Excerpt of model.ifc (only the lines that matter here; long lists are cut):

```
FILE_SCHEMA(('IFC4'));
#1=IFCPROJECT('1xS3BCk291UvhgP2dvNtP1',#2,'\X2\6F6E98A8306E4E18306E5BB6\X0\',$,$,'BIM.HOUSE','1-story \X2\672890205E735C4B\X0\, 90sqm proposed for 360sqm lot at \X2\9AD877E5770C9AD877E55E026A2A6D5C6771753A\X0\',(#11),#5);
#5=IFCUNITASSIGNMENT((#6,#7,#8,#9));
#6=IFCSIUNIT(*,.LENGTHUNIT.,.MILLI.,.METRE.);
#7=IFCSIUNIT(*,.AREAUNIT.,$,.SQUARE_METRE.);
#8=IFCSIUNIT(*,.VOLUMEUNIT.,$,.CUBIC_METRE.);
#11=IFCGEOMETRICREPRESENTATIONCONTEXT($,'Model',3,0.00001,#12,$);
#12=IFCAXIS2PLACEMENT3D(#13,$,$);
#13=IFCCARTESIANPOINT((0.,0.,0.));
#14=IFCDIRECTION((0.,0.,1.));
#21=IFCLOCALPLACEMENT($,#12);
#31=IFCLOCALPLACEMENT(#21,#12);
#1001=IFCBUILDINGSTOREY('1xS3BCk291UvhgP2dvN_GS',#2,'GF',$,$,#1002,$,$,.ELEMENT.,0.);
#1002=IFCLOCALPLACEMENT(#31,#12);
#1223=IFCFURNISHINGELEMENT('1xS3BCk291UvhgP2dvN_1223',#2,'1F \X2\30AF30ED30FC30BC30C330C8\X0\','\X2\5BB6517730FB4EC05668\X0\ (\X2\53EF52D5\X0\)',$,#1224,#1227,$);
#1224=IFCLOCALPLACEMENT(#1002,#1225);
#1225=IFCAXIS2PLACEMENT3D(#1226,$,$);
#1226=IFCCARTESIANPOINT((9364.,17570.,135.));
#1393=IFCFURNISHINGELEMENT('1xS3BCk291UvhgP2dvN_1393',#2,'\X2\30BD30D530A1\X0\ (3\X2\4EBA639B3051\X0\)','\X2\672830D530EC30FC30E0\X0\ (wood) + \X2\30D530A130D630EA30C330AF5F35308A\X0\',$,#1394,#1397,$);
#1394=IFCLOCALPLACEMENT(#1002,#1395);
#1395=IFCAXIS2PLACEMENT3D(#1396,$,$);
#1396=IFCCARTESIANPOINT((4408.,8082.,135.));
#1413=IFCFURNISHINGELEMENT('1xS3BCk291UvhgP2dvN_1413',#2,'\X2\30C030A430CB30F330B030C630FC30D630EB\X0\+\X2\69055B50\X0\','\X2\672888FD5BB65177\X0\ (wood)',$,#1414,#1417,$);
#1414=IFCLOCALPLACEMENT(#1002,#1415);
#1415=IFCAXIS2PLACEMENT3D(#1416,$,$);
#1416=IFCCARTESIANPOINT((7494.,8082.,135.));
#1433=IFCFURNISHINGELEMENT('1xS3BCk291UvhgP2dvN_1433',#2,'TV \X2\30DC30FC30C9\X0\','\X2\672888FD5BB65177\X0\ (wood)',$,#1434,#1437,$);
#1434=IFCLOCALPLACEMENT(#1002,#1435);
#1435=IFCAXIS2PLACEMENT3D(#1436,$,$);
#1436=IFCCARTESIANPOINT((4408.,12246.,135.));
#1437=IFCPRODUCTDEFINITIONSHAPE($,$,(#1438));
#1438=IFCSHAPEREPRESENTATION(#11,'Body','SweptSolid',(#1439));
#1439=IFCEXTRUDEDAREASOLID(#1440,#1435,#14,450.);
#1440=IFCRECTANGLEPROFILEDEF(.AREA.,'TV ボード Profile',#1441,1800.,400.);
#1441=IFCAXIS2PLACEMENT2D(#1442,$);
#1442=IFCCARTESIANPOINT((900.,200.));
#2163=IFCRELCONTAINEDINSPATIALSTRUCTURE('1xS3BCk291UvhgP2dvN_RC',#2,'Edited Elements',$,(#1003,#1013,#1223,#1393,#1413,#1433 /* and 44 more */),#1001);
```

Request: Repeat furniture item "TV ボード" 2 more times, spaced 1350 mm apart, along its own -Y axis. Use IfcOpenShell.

```python
import ifcopenshell
import ifcopenshell.api.geometry
import ifcopenshell.api.root
import ifcopenshell.util.element
import ifcopenshell.util.placement

model = ifcopenshell.open("model.ifc")


def reuse_history(source, copy):
    """copy_class also copies each property set's owner history, people and application; keep the originals."""
    for rel in copy.IsDefinedBy:
        if rel.is_a("IfcRelDefinesByProperties") and (history := rel.RelatingPropertyDefinition.OwnerHistory):
            rel.RelatingPropertyDefinition.OwnerHistory = source.OwnerHistory
            ifcopenshell.util.element.remove_deep2(model, history)


source = model.by_id(1433)
base = ifcopenshell.util.placement.get_local_placement(source.ObjectPlacement)
step = -base[:3, 1] * 1350.0

for i in range(1, 3):
    copy = ifcopenshell.api.root.copy_class(model, product=source)
    copy.Representation = ifcopenshell.util.element.copy_deep(
        model, source.Representation, exclude=["IfcGeometricRepresentationContext", "IfcRepresentationMap"]
    )
    reuse_history(source, copy)
    matrix = base.copy()
    matrix[:3, 3] += i * step
    print("added at", matrix[:3, 3].round(3) + 0.0)
    ifcopenshell.api.geometry.edit_object_placement(model, product=copy, matrix=matrix, is_si=False)

model.write("model_rev.ifc")
```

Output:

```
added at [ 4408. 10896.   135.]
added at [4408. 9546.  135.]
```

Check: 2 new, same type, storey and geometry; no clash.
